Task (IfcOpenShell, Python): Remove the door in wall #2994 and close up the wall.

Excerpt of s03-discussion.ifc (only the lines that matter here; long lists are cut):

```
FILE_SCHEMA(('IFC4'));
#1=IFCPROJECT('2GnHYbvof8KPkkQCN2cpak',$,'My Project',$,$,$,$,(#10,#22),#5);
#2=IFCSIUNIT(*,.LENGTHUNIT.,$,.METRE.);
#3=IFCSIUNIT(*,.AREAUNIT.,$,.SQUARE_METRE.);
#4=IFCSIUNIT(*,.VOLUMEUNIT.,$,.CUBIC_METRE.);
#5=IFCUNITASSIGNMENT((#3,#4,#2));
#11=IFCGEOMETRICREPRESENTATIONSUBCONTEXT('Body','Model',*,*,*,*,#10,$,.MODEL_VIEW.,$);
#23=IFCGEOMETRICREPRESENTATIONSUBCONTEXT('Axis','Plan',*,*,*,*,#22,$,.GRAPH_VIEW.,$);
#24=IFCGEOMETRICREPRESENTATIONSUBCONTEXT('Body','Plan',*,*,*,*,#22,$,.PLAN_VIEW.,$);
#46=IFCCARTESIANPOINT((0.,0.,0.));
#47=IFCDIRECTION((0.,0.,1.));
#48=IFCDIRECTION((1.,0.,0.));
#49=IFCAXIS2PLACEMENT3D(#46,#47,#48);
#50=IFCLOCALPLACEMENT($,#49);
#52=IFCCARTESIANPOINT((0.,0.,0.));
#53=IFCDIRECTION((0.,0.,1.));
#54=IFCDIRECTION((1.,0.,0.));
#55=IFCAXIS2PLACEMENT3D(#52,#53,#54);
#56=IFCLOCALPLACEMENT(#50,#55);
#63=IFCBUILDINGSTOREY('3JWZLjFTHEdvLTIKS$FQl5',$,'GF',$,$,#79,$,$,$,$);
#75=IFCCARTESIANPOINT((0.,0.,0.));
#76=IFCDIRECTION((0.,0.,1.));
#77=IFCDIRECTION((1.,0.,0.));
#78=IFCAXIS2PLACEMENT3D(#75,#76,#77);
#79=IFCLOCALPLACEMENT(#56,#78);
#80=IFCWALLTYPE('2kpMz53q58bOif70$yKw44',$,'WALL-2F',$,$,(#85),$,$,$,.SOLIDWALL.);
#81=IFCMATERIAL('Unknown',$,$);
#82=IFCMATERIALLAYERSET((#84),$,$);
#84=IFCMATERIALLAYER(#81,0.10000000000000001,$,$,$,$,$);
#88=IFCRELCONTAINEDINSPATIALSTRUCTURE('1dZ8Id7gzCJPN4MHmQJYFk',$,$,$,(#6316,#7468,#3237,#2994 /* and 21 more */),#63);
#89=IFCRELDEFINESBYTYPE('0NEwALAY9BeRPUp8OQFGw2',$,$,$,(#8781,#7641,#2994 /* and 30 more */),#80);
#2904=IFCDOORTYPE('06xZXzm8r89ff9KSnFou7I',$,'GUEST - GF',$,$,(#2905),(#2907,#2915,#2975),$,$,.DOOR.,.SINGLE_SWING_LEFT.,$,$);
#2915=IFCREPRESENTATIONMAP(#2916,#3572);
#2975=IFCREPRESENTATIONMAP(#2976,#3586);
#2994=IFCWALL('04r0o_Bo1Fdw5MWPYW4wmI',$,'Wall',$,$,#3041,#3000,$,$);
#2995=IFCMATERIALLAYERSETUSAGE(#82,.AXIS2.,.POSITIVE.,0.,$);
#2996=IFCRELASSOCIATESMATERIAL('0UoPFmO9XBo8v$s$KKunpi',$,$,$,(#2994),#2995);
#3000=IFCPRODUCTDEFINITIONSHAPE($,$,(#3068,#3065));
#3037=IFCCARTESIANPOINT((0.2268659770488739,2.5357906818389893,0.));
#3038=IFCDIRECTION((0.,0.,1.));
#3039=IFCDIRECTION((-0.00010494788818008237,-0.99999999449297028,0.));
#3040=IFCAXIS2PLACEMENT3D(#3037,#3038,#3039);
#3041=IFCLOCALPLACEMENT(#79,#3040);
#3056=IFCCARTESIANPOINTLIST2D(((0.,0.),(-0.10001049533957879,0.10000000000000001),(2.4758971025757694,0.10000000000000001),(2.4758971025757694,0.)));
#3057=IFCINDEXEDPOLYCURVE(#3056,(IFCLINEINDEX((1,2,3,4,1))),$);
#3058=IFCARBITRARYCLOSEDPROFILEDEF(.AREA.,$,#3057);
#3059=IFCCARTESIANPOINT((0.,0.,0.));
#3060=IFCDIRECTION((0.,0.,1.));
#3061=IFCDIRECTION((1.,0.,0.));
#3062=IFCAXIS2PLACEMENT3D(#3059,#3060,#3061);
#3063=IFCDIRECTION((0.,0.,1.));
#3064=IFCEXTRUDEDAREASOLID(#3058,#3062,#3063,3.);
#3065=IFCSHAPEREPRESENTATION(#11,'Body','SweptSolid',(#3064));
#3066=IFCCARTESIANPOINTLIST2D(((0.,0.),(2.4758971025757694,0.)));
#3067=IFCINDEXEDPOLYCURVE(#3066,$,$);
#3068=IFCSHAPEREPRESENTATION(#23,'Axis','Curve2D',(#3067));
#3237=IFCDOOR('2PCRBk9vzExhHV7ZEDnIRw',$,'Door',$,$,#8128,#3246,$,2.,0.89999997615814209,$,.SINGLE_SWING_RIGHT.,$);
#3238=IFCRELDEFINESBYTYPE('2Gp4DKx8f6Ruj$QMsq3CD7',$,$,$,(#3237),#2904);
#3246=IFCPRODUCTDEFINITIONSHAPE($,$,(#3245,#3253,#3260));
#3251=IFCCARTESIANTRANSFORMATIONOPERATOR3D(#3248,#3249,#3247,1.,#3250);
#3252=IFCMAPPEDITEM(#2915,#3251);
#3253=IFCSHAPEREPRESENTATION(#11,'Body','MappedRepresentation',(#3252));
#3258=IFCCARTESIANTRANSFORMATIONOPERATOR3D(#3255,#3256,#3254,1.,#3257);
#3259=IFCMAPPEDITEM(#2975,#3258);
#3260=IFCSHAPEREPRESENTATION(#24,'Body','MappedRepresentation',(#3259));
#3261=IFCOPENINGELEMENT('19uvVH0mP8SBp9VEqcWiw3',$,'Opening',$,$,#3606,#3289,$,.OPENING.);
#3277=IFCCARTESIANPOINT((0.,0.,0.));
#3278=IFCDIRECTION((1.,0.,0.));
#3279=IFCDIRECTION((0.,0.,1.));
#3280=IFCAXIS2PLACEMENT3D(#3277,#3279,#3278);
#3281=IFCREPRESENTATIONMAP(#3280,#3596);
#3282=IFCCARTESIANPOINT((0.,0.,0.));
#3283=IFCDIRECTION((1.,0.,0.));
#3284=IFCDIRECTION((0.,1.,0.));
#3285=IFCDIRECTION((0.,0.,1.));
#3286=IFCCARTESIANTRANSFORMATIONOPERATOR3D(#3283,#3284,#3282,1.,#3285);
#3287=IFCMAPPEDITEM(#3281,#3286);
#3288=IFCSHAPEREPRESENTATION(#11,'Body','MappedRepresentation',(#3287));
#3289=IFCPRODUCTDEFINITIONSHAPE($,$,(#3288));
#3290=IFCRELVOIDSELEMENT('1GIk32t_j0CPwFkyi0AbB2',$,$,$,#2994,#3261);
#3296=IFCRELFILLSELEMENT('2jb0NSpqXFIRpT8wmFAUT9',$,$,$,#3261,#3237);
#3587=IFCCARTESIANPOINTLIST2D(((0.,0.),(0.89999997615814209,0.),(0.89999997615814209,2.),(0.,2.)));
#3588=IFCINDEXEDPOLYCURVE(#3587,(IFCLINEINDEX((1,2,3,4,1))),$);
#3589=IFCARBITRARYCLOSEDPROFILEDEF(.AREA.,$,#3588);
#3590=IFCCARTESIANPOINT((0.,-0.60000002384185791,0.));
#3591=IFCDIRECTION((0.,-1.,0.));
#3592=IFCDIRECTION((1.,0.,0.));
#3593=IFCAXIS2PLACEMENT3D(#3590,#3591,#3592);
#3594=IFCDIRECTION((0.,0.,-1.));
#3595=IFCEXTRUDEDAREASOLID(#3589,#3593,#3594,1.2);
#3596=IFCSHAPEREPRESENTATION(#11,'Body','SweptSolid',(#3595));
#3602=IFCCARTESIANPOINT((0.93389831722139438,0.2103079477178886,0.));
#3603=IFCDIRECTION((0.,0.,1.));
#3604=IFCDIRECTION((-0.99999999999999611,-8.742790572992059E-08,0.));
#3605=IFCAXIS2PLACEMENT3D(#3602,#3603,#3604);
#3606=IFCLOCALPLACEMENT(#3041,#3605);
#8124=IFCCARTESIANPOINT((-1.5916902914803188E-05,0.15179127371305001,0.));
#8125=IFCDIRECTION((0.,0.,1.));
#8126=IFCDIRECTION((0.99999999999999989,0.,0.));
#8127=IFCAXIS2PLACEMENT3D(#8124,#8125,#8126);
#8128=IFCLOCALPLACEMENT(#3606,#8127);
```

```python
import ifcopenshell
import ifcopenshell.api.feature
import ifcopenshell.api.root
import ifcopenshell.geom
import ifcopenshell.util.shape

model = ifcopenshell.open("s03-discussion.ifc")
settings = ifcopenshell.geom.settings()


def volume(element):
    """Net volume in cubic metres, openings subtracted."""
    shape = ifcopenshell.geom.create_shape(settings, element)
    return ifcopenshell.util.shape.get_volume(shape.geometry)


door = model.by_guid("2PCRBk9vzExhHV7ZEDnIRw")
opening = door.FillsVoids[0].RelatingOpeningElement
wall = opening.VoidsElements[0].RelatingBuildingElement
before = volume(wall)

ifcopenshell.api.root.remove_product(model, product=door)
ifcopenshell.api.feature.remove_feature(model, feature=opening)

after = volume(wall)

print(f"wall volume {before:.3f} -> {after:.3f} m3")

model.write("s03-discussion_v2.ifc")
```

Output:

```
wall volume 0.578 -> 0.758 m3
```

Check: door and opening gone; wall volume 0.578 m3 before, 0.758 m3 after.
